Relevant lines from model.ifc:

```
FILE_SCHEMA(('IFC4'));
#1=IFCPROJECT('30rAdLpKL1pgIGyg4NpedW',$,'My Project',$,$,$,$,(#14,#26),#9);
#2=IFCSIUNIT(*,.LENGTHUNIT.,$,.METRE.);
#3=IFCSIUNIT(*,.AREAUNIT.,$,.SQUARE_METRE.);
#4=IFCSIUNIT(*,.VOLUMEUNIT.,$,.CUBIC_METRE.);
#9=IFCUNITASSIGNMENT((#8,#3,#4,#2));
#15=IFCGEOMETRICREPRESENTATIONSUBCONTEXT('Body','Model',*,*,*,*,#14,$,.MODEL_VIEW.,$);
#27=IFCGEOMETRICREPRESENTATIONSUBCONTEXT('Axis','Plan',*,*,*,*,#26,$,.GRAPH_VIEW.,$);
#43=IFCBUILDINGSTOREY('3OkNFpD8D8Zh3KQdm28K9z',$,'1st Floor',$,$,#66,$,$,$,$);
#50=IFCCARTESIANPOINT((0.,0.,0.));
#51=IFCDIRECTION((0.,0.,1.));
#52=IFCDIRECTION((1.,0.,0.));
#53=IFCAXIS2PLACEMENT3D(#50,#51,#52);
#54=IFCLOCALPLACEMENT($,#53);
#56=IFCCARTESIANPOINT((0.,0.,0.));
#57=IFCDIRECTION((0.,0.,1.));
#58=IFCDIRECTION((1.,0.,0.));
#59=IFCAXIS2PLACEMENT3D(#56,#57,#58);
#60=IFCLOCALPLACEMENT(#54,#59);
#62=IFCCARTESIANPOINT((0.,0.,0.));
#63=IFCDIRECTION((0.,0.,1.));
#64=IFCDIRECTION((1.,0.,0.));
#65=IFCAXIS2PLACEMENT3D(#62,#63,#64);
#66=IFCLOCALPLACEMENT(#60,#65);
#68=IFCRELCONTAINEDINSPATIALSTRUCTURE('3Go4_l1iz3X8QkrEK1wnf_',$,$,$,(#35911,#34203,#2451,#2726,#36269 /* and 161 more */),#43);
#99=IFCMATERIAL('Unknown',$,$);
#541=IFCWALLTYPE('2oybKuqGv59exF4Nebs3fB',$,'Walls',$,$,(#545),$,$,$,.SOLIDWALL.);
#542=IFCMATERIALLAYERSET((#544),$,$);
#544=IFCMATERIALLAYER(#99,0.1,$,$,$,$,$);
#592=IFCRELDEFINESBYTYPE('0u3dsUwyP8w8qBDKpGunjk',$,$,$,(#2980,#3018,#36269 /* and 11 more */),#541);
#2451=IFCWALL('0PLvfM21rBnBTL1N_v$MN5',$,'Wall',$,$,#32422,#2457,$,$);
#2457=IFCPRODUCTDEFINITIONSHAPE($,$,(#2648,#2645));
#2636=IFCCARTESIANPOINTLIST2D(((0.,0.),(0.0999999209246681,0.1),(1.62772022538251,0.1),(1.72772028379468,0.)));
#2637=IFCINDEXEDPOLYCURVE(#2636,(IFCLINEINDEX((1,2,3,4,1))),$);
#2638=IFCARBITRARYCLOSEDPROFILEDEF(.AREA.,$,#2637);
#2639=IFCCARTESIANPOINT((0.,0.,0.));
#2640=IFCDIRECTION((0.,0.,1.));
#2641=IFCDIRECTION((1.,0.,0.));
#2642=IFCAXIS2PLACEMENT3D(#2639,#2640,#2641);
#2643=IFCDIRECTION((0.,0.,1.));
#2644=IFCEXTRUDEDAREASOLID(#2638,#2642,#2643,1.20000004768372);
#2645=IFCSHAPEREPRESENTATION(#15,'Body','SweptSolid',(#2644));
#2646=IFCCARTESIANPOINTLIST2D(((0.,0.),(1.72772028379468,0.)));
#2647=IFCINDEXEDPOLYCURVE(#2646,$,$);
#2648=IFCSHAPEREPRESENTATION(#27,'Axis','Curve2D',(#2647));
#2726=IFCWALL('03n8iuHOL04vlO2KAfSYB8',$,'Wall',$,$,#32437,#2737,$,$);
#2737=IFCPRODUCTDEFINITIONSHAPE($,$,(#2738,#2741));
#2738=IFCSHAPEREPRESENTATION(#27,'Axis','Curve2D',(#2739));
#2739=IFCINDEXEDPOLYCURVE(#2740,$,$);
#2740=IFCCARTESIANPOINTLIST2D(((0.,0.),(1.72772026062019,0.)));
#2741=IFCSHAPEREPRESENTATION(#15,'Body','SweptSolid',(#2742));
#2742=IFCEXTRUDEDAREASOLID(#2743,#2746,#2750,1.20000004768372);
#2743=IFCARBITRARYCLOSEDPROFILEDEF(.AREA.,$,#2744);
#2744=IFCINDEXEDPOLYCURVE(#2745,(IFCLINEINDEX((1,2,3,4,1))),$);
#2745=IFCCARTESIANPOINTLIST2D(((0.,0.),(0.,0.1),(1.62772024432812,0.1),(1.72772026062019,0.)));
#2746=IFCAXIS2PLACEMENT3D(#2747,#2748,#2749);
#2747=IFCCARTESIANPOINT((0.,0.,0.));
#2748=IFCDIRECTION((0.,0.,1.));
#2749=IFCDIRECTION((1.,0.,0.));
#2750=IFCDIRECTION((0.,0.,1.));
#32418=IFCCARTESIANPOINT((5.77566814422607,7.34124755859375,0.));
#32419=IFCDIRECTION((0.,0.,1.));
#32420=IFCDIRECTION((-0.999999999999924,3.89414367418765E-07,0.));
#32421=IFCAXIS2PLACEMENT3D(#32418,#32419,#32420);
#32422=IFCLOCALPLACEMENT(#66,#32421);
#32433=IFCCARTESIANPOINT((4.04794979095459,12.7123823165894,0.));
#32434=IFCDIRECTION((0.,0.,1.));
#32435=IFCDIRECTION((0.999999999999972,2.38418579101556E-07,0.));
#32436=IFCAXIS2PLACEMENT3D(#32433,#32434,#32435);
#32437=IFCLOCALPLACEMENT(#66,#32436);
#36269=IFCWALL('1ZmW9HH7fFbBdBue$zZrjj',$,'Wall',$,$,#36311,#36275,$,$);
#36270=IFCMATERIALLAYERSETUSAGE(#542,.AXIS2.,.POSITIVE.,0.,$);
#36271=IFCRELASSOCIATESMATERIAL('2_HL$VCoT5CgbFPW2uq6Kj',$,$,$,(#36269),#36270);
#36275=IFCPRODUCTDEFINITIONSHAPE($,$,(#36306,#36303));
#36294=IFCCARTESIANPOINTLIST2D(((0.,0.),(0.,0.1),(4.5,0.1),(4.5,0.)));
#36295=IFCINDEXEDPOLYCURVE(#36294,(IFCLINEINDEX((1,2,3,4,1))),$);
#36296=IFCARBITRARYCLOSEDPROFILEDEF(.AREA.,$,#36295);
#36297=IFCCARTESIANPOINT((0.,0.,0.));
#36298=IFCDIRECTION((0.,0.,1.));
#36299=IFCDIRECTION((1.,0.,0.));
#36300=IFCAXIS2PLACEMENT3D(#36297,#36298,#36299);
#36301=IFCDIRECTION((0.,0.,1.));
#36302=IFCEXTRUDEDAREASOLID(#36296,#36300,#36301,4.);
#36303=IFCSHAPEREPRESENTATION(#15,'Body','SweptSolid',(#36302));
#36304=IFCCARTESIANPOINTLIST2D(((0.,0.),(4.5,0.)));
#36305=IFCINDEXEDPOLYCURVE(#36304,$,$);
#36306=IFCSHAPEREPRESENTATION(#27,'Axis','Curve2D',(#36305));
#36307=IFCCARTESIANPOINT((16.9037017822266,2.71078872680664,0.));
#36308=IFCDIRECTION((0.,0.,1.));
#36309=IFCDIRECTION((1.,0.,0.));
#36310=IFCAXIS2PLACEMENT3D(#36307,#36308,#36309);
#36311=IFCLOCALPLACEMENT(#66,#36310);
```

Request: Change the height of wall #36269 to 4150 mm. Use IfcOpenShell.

```python
import ifcopenshell
import ifcopenshell.geom
import ifcopenshell.util.representation
import ifcopenshell.util.shape
import ifcopenshell.util.unit

model = ifcopenshell.open("model.ifc")
unit_scale = ifcopenshell.util.unit.calculate_unit_scale(model)
settings = ifcopenshell.geom.settings()


def volume(element):
    """Net volume in cubic metres, openings subtracted."""
    shape = ifcopenshell.geom.create_shape(settings, element)
    return ifcopenshell.util.shape.get_volume(shape.geometry)


wall = model.by_guid("1ZmW9HH7fFbBdBue$zZrjj")
before = volume(wall)

body = ifcopenshell.util.representation.get_representation(wall, "Model", "Body")
solid = body.Items[0]
old_height = solid.Depth
solid.Depth = 4.15 / unit_scale
after = volume(wall)

print(f"height {old_height:g} -> {solid.Depth:g}, volume {before:.3f} -> {after:.3f} m3")

model.write("model_updated.ifc")
```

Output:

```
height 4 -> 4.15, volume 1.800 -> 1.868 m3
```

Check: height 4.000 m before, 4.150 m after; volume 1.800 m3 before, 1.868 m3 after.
